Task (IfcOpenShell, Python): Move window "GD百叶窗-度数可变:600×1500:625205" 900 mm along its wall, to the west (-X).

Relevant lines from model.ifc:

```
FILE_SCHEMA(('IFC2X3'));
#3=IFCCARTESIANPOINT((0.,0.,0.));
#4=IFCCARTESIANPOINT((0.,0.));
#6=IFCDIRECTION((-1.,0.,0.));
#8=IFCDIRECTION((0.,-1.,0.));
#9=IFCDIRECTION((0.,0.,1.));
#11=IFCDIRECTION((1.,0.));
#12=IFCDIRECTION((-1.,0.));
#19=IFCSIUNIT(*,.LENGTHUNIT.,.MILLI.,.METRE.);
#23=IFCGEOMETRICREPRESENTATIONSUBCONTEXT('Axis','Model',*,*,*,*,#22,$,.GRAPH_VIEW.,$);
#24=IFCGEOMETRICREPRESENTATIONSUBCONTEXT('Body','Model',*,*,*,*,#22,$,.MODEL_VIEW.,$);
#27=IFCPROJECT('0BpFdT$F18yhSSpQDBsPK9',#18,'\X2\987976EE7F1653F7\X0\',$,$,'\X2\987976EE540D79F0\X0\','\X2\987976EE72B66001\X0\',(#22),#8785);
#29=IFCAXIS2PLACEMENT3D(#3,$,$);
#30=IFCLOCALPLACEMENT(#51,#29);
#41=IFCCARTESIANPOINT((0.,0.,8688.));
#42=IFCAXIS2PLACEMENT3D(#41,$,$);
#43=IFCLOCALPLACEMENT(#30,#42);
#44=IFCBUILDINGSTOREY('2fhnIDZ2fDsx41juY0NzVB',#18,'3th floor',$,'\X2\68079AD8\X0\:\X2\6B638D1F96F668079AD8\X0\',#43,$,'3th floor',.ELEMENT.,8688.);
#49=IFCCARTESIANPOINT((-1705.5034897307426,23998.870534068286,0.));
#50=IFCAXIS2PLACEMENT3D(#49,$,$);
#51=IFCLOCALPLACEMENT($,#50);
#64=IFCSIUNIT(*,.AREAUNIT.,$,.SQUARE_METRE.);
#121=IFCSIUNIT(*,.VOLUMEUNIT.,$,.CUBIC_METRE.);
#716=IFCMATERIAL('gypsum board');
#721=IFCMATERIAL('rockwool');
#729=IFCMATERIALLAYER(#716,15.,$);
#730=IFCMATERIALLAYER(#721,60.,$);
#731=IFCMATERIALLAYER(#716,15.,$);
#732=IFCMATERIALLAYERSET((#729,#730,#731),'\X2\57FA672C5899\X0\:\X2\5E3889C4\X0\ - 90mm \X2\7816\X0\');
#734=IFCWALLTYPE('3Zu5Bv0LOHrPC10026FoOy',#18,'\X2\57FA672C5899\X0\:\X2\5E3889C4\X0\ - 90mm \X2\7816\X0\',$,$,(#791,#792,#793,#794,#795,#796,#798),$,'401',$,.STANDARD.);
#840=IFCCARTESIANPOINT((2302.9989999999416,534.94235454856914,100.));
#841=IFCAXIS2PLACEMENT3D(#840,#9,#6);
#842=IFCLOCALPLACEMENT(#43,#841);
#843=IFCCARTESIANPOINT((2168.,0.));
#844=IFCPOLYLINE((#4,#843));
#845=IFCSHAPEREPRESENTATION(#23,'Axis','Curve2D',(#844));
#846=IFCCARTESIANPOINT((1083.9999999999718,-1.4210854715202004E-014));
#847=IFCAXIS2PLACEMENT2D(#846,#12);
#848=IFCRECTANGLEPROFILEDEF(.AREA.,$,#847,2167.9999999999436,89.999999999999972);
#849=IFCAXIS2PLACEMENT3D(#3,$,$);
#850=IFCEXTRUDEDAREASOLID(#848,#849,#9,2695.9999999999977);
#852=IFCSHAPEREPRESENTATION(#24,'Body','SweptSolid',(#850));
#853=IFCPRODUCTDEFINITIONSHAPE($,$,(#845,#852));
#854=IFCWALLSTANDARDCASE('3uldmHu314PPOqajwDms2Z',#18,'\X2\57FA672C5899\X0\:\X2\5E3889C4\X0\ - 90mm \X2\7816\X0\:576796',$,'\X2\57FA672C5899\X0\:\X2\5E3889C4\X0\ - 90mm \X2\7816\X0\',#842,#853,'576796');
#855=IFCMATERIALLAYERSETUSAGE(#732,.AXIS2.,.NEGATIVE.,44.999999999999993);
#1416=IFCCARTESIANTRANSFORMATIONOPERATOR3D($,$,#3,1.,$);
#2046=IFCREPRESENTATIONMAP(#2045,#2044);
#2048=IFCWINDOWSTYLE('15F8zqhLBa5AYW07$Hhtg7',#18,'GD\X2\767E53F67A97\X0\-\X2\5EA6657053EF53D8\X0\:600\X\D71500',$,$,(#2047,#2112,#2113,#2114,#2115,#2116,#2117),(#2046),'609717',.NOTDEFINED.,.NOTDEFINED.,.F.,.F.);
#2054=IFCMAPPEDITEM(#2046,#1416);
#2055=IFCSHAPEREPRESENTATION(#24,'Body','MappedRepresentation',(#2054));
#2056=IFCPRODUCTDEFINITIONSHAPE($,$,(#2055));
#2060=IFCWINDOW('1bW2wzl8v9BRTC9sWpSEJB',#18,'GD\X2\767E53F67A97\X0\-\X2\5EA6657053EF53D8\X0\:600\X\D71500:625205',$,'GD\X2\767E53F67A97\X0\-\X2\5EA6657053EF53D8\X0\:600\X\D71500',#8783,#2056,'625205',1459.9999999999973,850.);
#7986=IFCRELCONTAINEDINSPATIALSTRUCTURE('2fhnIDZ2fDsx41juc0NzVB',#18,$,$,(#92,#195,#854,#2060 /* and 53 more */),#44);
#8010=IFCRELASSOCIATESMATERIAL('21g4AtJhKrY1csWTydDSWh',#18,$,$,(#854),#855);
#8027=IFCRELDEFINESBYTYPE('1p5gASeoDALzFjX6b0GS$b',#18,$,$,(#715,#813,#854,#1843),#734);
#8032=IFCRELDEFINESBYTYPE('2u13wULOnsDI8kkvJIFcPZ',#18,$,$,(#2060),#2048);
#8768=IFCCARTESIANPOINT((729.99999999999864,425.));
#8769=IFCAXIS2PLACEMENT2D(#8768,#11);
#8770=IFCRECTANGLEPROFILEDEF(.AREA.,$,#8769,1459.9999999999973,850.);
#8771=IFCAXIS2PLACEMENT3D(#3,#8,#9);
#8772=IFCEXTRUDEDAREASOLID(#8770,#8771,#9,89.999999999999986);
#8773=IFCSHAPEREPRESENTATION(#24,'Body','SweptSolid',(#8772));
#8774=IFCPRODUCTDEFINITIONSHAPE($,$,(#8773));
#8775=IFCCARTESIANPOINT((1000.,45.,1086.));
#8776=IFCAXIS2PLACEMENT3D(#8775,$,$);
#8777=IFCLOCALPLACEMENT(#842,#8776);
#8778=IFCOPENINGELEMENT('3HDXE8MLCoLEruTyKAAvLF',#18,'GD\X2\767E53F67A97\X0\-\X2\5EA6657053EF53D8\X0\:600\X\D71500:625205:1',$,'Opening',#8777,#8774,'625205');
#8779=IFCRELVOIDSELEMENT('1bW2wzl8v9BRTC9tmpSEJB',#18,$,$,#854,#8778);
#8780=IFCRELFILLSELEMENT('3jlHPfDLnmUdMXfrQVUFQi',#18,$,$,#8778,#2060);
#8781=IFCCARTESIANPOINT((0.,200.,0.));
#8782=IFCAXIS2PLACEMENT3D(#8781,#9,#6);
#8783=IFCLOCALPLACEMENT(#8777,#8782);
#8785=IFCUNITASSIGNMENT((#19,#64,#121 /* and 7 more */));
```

```python
import ifcopenshell
import ifcopenshell.api.geometry
import ifcopenshell.util.placement

model = ifcopenshell.open("model.ifc")

window = model.by_guid("1bW2wzl8v9BRTC9sWpSEJB")
opening = window.FillsVoids[0].RelatingOpeningElement
wall = opening.VoidsElements[0].RelatingBuildingElement

wall_matrix = ifcopenshell.util.placement.get_local_placement(wall.ObjectPlacement)
shift = wall_matrix[:3, 0] * 900.0
before = ifcopenshell.util.placement.get_local_placement(window.ObjectPlacement)[:3, 3].copy()

# The window is placed relative to its opening, so it follows when the opening moves.
matrix = ifcopenshell.util.placement.get_local_placement(opening.ObjectPlacement)
matrix[:3, 3] += shift
ifcopenshell.api.geometry.edit_object_placement(
    model, product=opening, matrix=matrix, is_si=False, should_transform_children=True
)

after = ifcopenshell.util.placement.get_local_placement(window.ObjectPlacement)[:3, 3]
print("window moved by", (after - before).round(3) + 0.0)

model.write("model_edited.ifc")
```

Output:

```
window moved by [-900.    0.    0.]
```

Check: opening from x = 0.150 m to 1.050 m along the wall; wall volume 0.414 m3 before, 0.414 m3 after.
